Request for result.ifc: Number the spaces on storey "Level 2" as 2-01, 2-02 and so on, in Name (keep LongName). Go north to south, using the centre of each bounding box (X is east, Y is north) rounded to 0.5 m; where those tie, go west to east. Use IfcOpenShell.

First a look at what the model holds.

```python
import ifcopenshell
import ifcopenshell.util.element
import ifcopenshell.util.placement

model = ifcopenshell.open("result.ifc")
print(model.schema)
storey = next(s for s in model.by_type("IfcBuildingStorey") if s.Name == "Level 2")
spaces = [e for e in ifcopenshell.util.element.get_decomposition(storey) if e.is_a("IfcSpace")]
for e in sorted(spaces, key=lambda e: e.id()):
    origin = ifcopenshell.util.placement.get_local_placement(e.ObjectPlacement)[:3, 3]
    print(e.id(), e.Name, e.LongName, origin.round(2) + 0.0, sep=" | ")
```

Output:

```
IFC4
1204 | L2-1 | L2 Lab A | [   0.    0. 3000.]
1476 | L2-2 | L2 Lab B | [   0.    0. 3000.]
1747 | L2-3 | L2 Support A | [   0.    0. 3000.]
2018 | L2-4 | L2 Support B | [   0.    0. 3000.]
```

```python
import ifcopenshell
import ifcopenshell.geom
import ifcopenshell.util.element
import ifcopenshell.util.shape

model = ifcopenshell.open("result.ifc")
settings = ifcopenshell.geom.settings()
settings.set("use-world-coords", True)


def centre(element):
    shape = ifcopenshell.geom.create_shape(settings, element)
    return ifcopenshell.util.shape.get_bbox_centroid(shape.geometry)


storey = next(s for s in model.by_type("IfcBuildingStorey") if s.Name == "Level 2")
spaces = [e for e in ifcopenshell.util.element.get_decomposition(storey) if e.is_a("IfcSpace")]

# Insertion points can sit at a corner or the storey origin, so sort by the geometry (in metres).
centres = {e: centre(e) for e in spaces}
spaces.sort(key=lambda e: (-round(centres[e][1] / 0.5), centres[e][0]))

for i, e in enumerate(spaces, start=1):
    number = f"2-{i:02d}"
    e.Name = number
    print(e.id(), number)

model.write("result_rev.ifc")
```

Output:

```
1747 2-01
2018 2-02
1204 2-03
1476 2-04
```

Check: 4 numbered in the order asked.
